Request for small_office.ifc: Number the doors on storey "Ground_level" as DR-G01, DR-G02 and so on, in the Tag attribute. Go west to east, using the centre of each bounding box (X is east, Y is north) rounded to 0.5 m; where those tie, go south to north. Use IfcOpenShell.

First a look at what the model holds.

```python
import ifcopenshell
import ifcopenshell.util.element
import ifcopenshell.util.placement

model = ifcopenshell.open("small_office.ifc")
print(model.schema)
storey = next(s for s in model.by_type("IfcBuildingStorey") if s.Name == "Ground_level")
doors = [e for e in ifcopenshell.util.element.get_decomposition(storey) if e.is_a("IfcDoor")]
for e in sorted(doors, key=lambda e: e.id()):
    origin = ifcopenshell.util.placement.get_local_placement(e.ObjectPlacement)[:3, 3]
    print(e.id(), e.Tag, e.Name, origin.round(2) + 0.0, sep=" | ")
```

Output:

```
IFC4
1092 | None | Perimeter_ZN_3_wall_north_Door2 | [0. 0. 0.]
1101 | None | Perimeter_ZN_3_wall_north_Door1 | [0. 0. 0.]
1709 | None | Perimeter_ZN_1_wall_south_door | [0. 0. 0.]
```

```python
import ifcopenshell
import ifcopenshell.geom
import ifcopenshell.util.element
import ifcopenshell.util.shape

model = ifcopenshell.open("small_office.ifc")
settings = ifcopenshell.geom.settings()
settings.set("use-world-coords", True)


def centre(element):
    shape = ifcopenshell.geom.create_shape(settings, element)
    return ifcopenshell.util.shape.get_bbox_centroid(shape.geometry)


storey = next(s for s in model.by_type("IfcBuildingStorey") if s.Name == "Ground_level")
doors = [e for e in ifcopenshell.util.element.get_decomposition(storey) if e.is_a("IfcDoor")]

# Insertion points can sit at a corner or the storey origin, so sort by the geometry (in metres).
centres = {e: centre(e) for e in doors}
doors.sort(key=lambda e: (round(centres[e][0] / 0.5), centres[e][1]))

for i, e in enumerate(doors, start=1):
    number = f"DR-G{i:02d}"
    e.Tag = number
    print(e.id(), number)

model.write("small_office_v2.ifc")
```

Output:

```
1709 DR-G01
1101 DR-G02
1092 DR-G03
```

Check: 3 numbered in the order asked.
